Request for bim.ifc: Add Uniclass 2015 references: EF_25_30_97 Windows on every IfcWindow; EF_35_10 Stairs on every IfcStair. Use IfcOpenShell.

First a look at what the model holds.

```python
import ifcopenshell

model = ifcopenshell.open("bim.ifc")
print(model.schema)
print("classifications:", [c.Name for c in model.by_type("IfcClassification")])
for ifc_class in ("IfcDoor", "IfcRoof", "IfcStair", "IfcWall", "IfcWindow"):
    print(ifc_class, len(model.by_type(ifc_class)))
```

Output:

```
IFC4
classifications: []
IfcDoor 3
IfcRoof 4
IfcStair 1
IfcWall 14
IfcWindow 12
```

```python
import ifcopenshell
import ifcopenshell.api.classification

model = ifcopenshell.open("bim.ifc")

system = ifcopenshell.api.classification.add_classification(model, classification="Uniclass 2015")

codes = {
    "IfcWindow": ("EF_25_30_97", "Windows"),
    "IfcStair": ("EF_35_10", "Stairs"),
}
for ifc_class, (code, name) in codes.items():
    products = model.by_type(ifc_class)
    ifcopenshell.api.classification.add_reference(
        model, products=products, classification=system, identification=code, name=name
    )
    print(code, len(products))

model.write("bim_rev.ifc")
```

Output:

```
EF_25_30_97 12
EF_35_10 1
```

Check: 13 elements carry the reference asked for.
